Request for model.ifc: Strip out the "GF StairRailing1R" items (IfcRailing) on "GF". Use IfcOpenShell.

First a look at what the model holds.

```python
import ifcopenshell
import ifcopenshell.util.element

model = ifcopenshell.open("model.ifc")
print(model.schema)
storey = next(s for s in model.by_type("IfcBuildingStorey") if s.Name == "GF")
railings = [e for e in ifcopenshell.util.element.get_decomposition(storey) if e.is_a("IfcRailing")]
seen = {}
for e in railings:
    element_type = ifcopenshell.util.element.get_type(e)
    name = element_type.Name if element_type not in (None, e) else None
    seen[name] = seen.get(name, 0) + 1
for name, count in sorted(seen.items(), key=str):
    print(count, "x", name)
```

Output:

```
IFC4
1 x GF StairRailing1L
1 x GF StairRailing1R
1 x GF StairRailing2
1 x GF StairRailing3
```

```python
import ifcopenshell
import ifcopenshell.api.root
import ifcopenshell.util.element

model = ifcopenshell.open("model.ifc")

storey = next(s for s in model.by_type("IfcBuildingStorey") if s.Name == "GF")
railings = [e for e in ifcopenshell.util.element.get_decomposition(storey) if e.is_a("IfcRailing")]
targets = [e for e in railings if (t := ifcopenshell.util.element.get_type(e)) not in (None, e) and t.Name == "GF StairRailing1R"]

for e in targets:
    ifcopenshell.api.root.remove_product(model, product=e)
print(len(targets), "removed")

model.write("model-out.ifc")
```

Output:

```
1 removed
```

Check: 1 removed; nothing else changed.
